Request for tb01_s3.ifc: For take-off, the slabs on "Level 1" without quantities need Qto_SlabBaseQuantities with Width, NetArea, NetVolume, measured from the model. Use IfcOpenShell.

First a look at what the model holds.

```python
import ifcopenshell
import ifcopenshell.util.element
import ifcopenshell.util.unit

model = ifcopenshell.open("tb01_s3.ifc")
print(model.schema)
for unit_type in ("LENGTHUNIT", "AREAUNIT", "VOLUMEUNIT"):
    print(unit_type, ifcopenshell.util.unit.calculate_unit_scale(model, unit_type))
storey = next(s for s in model.by_type("IfcBuildingStorey") if s.Name == "Level 1")
slabs = [e for e in ifcopenshell.util.element.get_decomposition(storey) if e.is_a("IfcSlab")]
for e in sorted(slabs, key=lambda e: e.id()):
    print(e.id(), e.is_a(), e.Name, list(ifcopenshell.util.element.get_psets(e, qtos_only=True)), sep=" | ")
```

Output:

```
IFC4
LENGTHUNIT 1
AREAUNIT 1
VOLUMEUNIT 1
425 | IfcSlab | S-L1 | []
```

```python
import ifcopenshell
import ifcopenshell.api.pset
import ifcopenshell.geom
import ifcopenshell.util.element
import ifcopenshell.util.shape
import ifcopenshell.util.unit

model = ifcopenshell.open("tb01_s3.ifc")
unit_scale = ifcopenshell.util.unit.calculate_unit_scale(model)
area_scale = ifcopenshell.util.unit.calculate_unit_scale(model, "AREAUNIT")
volume_scale = ifcopenshell.util.unit.calculate_unit_scale(model, "VOLUMEUNIT")
settings = ifcopenshell.geom.settings()

storey = next(s for s in model.by_type("IfcBuildingStorey") if s.Name == "Level 1")
slabs = [e for e in ifcopenshell.util.element.get_decomposition(storey) if e.is_a("IfcSlab")]

for e in sorted(slabs, key=lambda e: e.id()):
    if ifcopenshell.util.element.get_psets(e, qtos_only=True, should_inherit=False):
        continue
    # Geometry comes back in metres, in the element's own axes.
    shape = ifcopenshell.geom.create_shape(settings, e)
    values = {
        "Width": ifcopenshell.util.shape.get_z(shape.geometry) / unit_scale,
        "NetArea": ifcopenshell.util.shape.get_footprint_area(shape.geometry) / area_scale,
        "NetVolume": ifcopenshell.util.shape.get_volume(shape.geometry) / volume_scale,
    }
    qto = ifcopenshell.api.pset.add_qto(model, product=e, name="Qto_SlabBaseQuantities")
    ifcopenshell.api.pset.edit_qto(model, qto=qto, properties=values)
    print(e.id(), {k: round(v, 3) for k, v in values.items()})

model.write("tb01_s3_rev.ifc")
```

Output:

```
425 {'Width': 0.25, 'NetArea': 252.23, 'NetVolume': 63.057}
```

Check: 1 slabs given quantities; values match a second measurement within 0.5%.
